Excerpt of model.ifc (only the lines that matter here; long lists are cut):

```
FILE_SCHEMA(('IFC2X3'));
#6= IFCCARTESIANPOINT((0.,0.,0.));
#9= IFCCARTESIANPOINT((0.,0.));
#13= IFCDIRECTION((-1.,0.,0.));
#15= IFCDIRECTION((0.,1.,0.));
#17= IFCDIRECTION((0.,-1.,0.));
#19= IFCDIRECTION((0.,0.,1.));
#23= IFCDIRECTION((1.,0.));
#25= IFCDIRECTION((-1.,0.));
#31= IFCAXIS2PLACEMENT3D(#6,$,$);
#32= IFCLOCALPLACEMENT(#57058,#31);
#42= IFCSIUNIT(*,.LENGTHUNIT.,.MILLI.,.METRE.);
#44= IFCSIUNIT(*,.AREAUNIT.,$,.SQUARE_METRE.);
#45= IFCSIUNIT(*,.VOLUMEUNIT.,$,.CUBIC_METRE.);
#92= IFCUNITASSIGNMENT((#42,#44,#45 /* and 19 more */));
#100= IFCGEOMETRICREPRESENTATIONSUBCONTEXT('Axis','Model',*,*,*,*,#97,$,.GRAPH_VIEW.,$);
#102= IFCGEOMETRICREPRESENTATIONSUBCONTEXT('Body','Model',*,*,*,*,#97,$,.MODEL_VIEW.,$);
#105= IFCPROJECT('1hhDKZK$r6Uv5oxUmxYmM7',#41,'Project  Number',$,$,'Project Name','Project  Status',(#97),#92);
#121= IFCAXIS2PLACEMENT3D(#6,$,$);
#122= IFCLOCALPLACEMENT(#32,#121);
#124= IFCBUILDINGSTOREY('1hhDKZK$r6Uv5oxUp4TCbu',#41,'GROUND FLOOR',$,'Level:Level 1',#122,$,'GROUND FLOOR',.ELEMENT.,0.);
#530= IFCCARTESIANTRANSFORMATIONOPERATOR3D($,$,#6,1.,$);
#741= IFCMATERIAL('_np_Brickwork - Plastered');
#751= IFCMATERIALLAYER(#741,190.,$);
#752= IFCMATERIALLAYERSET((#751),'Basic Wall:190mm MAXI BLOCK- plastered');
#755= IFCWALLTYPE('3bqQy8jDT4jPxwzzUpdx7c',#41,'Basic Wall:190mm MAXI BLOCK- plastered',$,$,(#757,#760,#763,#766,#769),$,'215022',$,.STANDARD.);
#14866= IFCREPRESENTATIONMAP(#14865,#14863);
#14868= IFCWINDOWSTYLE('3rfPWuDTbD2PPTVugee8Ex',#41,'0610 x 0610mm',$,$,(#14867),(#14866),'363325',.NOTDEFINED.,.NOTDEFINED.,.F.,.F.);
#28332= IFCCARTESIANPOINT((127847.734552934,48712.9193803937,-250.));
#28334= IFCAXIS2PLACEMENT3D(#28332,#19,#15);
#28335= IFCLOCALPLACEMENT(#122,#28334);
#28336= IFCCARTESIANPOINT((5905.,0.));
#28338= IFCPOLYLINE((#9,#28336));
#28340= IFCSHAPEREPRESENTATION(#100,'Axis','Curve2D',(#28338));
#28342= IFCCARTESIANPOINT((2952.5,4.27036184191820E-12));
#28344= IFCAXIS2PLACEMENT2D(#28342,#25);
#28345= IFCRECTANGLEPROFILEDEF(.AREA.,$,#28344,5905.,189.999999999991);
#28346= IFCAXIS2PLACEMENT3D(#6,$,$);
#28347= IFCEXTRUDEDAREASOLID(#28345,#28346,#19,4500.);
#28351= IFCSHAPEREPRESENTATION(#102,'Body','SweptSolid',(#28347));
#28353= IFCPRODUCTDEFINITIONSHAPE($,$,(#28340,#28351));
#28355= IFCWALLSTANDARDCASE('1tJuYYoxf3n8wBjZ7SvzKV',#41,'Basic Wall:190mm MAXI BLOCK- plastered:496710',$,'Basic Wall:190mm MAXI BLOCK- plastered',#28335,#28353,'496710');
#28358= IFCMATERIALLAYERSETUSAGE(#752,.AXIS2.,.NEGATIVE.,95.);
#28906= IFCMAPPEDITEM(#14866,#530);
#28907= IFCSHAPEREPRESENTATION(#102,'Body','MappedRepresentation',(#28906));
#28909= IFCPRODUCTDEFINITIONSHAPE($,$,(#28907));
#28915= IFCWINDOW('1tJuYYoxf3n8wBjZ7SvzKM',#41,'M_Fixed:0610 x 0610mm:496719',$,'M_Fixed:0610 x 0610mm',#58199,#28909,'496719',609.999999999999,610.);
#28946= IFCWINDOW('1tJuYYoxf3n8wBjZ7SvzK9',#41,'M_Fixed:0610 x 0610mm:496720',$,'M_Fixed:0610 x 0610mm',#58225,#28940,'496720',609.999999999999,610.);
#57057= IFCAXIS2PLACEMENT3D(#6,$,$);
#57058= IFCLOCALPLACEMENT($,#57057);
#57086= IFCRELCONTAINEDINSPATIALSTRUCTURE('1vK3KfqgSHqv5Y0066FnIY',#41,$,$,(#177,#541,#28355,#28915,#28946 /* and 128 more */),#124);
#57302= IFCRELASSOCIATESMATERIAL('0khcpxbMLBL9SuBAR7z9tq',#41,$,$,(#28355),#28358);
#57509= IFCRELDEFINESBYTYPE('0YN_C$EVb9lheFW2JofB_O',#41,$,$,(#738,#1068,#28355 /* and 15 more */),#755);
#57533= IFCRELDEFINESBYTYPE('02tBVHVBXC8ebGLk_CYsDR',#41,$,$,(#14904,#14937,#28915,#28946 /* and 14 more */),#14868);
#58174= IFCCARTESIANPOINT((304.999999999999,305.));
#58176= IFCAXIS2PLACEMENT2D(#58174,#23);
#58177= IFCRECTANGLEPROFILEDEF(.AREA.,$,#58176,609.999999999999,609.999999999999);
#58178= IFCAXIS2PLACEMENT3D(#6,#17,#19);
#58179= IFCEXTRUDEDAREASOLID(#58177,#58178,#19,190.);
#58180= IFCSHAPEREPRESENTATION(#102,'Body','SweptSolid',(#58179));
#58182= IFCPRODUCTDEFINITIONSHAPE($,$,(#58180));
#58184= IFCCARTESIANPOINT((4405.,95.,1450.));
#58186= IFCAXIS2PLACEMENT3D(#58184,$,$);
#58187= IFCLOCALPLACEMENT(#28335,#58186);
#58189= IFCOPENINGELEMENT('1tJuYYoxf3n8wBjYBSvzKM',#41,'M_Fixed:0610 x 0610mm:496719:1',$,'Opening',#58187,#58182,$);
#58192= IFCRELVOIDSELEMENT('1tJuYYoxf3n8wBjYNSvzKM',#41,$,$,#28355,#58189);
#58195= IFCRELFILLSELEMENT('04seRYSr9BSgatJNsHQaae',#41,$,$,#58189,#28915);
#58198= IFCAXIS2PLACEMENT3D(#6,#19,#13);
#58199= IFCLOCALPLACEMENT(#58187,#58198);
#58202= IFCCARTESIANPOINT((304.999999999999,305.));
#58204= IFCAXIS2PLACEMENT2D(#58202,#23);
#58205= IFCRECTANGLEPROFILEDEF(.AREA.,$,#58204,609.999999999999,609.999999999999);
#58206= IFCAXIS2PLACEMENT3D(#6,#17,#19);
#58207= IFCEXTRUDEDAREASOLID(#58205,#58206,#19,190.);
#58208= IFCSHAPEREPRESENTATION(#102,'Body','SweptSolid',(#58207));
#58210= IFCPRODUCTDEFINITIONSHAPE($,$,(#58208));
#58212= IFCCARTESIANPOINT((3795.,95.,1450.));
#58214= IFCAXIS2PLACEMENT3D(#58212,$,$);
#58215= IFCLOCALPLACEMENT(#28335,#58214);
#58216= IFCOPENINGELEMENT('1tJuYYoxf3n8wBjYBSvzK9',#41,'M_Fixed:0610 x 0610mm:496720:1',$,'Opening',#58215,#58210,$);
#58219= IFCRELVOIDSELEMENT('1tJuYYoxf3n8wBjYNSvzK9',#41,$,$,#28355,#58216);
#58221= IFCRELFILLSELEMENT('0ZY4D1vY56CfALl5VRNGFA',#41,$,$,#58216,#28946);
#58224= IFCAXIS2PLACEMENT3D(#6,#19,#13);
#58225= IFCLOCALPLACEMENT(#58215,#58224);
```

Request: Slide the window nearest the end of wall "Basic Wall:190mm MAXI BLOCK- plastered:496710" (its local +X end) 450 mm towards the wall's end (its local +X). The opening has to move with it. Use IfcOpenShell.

```python
import ifcopenshell
import ifcopenshell.api.geometry
import ifcopenshell.util.placement
import ifcopenshell.util.unit

model = ifcopenshell.open("model.ifc")
unit_scale = ifcopenshell.util.unit.calculate_unit_scale(model)

window = model.by_id(28915)
opening = window.FillsVoids[0].RelatingOpeningElement
wall = opening.VoidsElements[0].RelatingBuildingElement

wall_matrix = ifcopenshell.util.placement.get_local_placement(wall.ObjectPlacement)
shift = wall_matrix[:3, 0] * 0.45 / unit_scale
before = ifcopenshell.util.placement.get_local_placement(window.ObjectPlacement)[:3, 3].copy()

# The window is placed relative to its opening, so it follows when the opening moves.
matrix = ifcopenshell.util.placement.get_local_placement(opening.ObjectPlacement)
matrix[:3, 3] += shift
ifcopenshell.api.geometry.edit_object_placement(
    model, product=opening, matrix=matrix, is_si=False, should_transform_children=True
)

after = ifcopenshell.util.placement.get_local_placement(window.ObjectPlacement)[:3, 3]
print("window moved by", (after - before).round(3) + 0.0)

model.write("model_updated.ifc")
```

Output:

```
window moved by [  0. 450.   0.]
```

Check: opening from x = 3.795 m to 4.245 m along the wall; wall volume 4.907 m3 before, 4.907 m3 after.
